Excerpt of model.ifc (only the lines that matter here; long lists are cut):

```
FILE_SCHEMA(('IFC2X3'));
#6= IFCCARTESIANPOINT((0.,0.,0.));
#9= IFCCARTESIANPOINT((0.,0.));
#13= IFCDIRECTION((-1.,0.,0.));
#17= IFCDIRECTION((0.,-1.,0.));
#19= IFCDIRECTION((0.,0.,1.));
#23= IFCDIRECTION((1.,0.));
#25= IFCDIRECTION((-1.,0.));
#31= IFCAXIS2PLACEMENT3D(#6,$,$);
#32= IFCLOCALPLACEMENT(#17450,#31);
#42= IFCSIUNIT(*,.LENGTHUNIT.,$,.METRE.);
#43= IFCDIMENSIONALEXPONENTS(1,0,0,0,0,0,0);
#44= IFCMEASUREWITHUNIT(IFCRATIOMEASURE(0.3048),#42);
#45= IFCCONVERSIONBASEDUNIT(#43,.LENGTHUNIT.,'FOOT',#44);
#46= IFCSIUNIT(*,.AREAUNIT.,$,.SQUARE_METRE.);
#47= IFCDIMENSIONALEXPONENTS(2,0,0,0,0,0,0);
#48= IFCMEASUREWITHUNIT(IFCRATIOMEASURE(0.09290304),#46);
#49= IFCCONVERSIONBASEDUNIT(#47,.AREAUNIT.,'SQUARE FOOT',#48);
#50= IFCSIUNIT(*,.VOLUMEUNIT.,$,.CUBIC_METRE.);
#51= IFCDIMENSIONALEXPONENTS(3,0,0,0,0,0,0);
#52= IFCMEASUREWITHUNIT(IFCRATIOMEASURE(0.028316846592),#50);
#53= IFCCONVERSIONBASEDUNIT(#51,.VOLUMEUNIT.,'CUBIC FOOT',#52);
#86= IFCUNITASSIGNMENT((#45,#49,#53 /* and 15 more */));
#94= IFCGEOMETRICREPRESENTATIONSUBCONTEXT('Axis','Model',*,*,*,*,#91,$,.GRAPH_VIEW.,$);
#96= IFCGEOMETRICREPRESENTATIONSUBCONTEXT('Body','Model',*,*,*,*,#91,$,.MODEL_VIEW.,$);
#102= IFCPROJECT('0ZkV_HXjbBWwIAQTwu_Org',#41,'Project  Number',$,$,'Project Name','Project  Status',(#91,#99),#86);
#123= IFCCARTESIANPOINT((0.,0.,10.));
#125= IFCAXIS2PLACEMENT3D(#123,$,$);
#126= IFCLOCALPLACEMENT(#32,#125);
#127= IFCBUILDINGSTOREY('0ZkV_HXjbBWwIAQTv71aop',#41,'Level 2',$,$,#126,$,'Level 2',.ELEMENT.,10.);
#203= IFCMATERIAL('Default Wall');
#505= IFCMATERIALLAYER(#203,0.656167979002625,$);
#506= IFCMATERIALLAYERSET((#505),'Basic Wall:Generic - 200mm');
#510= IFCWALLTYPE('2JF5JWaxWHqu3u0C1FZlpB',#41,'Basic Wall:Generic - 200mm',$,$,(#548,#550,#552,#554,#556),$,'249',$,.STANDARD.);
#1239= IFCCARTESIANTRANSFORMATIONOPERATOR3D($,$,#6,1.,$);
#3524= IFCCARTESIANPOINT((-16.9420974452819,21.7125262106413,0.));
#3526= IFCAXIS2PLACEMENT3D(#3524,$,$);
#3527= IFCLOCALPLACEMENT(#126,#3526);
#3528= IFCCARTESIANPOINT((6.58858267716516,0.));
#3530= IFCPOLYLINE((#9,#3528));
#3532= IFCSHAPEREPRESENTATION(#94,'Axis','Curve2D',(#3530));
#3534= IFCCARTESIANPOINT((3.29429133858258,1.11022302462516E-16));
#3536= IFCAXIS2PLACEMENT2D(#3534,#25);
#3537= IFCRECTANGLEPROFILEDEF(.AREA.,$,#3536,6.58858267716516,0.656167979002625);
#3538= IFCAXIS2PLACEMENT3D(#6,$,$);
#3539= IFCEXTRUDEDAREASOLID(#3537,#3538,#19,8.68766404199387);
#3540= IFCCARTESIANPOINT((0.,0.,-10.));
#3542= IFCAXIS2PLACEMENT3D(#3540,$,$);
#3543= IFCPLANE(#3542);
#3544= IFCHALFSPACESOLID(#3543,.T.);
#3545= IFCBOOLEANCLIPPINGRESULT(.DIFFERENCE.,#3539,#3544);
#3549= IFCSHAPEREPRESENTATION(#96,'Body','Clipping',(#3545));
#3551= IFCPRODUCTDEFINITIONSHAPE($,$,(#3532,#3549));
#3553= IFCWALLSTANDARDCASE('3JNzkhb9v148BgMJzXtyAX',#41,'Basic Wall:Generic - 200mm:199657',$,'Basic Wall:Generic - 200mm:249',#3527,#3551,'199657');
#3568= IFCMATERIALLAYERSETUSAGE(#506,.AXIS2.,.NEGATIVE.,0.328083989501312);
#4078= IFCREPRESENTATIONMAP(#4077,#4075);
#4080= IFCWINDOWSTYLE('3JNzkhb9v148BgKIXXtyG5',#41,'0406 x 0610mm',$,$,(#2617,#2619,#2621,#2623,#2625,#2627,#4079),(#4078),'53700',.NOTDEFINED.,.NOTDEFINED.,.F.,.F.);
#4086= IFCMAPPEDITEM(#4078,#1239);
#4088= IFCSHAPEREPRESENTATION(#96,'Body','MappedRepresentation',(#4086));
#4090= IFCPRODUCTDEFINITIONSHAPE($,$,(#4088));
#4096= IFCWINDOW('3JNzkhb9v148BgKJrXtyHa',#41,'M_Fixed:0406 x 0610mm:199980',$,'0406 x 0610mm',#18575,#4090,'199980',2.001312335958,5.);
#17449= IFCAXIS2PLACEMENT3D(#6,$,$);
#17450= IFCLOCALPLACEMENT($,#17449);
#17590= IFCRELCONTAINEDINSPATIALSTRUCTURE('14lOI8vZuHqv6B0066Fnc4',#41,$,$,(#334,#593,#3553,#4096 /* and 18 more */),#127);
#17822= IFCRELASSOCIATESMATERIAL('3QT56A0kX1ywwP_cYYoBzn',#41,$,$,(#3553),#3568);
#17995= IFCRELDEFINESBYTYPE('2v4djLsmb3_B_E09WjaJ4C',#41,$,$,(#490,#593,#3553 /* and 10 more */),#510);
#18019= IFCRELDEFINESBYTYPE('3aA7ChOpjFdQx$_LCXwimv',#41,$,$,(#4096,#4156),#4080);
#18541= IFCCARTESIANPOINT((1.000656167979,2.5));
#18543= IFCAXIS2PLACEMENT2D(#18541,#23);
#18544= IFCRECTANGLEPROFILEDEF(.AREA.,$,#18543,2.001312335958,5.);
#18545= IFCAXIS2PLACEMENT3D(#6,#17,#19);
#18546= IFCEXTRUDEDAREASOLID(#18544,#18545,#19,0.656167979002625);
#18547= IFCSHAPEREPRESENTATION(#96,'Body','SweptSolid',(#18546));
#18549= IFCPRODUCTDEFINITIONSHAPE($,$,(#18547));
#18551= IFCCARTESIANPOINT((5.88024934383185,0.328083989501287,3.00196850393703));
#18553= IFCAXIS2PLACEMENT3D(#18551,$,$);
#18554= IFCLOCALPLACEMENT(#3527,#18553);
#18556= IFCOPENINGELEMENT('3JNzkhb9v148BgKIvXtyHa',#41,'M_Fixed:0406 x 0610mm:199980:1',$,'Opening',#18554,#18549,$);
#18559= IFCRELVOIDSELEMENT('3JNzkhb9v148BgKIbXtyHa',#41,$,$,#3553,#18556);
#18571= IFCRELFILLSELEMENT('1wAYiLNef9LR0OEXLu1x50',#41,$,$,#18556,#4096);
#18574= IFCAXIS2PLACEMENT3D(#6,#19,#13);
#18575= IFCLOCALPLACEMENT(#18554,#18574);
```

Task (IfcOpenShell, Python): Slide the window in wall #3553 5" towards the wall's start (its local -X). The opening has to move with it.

```python
import ifcopenshell
import ifcopenshell.api.geometry
import ifcopenshell.util.placement
import ifcopenshell.util.unit

model = ifcopenshell.open("model.ifc")
unit_scale = ifcopenshell.util.unit.calculate_unit_scale(model)

window = model.by_guid("3JNzkhb9v148BgKJrXtyHa")
opening = window.FillsVoids[0].RelatingOpeningElement
wall = opening.VoidsElements[0].RelatingBuildingElement

wall_matrix = ifcopenshell.util.placement.get_local_placement(wall.ObjectPlacement)
shift = wall_matrix[:3, 0] * -5 * 0.0254 / unit_scale
before = ifcopenshell.util.placement.get_local_placement(window.ObjectPlacement)[:3, 3].copy()

# The window is placed relative to its opening, so it follows when the opening moves.
matrix = ifcopenshell.util.placement.get_local_placement(opening.ObjectPlacement)
matrix[:3, 3] += shift
ifcopenshell.api.geometry.edit_object_placement(
    model, product=opening, matrix=matrix, is_si=False, should_transform_children=True
)

after = ifcopenshell.util.placement.get_local_placement(window.ObjectPlacement)[:3, 3]
print("window moved by", (after - before).round(3) + 0.0)

model.write("model-out.ifc")
```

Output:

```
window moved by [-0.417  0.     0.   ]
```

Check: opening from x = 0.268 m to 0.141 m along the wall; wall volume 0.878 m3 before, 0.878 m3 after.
